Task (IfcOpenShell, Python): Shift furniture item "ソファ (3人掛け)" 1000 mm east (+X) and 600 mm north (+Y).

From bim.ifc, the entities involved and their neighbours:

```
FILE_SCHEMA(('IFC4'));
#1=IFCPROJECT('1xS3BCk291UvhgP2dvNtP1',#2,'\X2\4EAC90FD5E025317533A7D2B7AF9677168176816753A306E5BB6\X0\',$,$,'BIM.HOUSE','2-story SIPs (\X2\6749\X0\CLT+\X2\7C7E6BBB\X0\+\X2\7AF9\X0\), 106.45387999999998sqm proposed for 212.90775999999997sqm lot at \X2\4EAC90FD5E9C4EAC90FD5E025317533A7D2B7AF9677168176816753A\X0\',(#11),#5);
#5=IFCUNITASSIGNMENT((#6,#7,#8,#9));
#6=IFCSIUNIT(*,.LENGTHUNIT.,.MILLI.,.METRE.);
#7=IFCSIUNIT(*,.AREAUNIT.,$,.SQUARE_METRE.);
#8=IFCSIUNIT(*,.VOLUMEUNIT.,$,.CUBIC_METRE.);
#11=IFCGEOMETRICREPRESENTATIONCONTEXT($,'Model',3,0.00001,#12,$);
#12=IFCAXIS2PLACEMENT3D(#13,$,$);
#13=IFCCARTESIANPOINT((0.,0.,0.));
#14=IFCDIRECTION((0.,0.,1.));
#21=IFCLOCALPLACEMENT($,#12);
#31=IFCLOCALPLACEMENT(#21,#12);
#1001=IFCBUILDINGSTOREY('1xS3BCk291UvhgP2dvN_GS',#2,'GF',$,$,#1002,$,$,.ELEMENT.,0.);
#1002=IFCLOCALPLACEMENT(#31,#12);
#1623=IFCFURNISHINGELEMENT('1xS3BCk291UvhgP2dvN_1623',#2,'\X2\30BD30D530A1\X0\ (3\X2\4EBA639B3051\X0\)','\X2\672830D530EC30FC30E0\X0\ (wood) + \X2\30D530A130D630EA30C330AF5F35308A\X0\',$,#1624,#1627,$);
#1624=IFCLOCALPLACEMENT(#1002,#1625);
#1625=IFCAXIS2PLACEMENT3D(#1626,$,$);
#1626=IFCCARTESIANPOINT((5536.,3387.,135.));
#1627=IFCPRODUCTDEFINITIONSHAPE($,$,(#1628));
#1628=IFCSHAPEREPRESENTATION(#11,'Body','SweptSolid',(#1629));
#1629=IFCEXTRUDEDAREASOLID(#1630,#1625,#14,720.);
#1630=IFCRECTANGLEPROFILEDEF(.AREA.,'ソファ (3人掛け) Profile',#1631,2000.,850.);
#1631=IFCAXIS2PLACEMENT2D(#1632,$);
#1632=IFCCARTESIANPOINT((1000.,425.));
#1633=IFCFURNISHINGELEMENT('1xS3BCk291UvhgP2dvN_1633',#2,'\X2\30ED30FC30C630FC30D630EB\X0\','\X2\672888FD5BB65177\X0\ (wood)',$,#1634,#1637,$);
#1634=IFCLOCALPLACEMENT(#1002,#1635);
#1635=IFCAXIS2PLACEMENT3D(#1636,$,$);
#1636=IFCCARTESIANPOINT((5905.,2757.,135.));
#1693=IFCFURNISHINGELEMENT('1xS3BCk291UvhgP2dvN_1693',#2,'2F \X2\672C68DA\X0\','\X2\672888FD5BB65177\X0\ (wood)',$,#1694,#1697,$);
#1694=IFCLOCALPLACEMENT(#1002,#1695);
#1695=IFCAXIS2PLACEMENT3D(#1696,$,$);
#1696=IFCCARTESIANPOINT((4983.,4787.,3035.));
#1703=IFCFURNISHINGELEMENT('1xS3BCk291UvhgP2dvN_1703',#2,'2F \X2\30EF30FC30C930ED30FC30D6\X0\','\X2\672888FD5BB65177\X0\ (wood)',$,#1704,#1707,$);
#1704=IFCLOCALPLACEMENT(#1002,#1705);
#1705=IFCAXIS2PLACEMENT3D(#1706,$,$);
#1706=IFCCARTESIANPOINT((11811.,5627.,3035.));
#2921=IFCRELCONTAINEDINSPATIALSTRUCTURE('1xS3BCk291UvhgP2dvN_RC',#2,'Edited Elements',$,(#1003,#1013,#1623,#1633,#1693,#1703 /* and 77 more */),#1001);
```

```python
import ifcopenshell
import ifcopenshell.api.geometry
import ifcopenshell.util.placement
import ifcopenshell.util.unit

model = ifcopenshell.open("bim.ifc")
unit_scale = ifcopenshell.util.unit.calculate_unit_scale(model)

item = model.by_id(1623)
matrix = ifcopenshell.util.placement.get_local_placement(item.ObjectPlacement)
matrix[0, 3] += 1 / unit_scale
matrix[1, 3] += 0.6 / unit_scale
ifcopenshell.api.geometry.edit_object_placement(model, product=item, matrix=matrix, is_si=False)

print(ifcopenshell.util.placement.get_local_placement(item.ObjectPlacement).round(3) + 0.0)

model.write("bim_edited.ifc")
```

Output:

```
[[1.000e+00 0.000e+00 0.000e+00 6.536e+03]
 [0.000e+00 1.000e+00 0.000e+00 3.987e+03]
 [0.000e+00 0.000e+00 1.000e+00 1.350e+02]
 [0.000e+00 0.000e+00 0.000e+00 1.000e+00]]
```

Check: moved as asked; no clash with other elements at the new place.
